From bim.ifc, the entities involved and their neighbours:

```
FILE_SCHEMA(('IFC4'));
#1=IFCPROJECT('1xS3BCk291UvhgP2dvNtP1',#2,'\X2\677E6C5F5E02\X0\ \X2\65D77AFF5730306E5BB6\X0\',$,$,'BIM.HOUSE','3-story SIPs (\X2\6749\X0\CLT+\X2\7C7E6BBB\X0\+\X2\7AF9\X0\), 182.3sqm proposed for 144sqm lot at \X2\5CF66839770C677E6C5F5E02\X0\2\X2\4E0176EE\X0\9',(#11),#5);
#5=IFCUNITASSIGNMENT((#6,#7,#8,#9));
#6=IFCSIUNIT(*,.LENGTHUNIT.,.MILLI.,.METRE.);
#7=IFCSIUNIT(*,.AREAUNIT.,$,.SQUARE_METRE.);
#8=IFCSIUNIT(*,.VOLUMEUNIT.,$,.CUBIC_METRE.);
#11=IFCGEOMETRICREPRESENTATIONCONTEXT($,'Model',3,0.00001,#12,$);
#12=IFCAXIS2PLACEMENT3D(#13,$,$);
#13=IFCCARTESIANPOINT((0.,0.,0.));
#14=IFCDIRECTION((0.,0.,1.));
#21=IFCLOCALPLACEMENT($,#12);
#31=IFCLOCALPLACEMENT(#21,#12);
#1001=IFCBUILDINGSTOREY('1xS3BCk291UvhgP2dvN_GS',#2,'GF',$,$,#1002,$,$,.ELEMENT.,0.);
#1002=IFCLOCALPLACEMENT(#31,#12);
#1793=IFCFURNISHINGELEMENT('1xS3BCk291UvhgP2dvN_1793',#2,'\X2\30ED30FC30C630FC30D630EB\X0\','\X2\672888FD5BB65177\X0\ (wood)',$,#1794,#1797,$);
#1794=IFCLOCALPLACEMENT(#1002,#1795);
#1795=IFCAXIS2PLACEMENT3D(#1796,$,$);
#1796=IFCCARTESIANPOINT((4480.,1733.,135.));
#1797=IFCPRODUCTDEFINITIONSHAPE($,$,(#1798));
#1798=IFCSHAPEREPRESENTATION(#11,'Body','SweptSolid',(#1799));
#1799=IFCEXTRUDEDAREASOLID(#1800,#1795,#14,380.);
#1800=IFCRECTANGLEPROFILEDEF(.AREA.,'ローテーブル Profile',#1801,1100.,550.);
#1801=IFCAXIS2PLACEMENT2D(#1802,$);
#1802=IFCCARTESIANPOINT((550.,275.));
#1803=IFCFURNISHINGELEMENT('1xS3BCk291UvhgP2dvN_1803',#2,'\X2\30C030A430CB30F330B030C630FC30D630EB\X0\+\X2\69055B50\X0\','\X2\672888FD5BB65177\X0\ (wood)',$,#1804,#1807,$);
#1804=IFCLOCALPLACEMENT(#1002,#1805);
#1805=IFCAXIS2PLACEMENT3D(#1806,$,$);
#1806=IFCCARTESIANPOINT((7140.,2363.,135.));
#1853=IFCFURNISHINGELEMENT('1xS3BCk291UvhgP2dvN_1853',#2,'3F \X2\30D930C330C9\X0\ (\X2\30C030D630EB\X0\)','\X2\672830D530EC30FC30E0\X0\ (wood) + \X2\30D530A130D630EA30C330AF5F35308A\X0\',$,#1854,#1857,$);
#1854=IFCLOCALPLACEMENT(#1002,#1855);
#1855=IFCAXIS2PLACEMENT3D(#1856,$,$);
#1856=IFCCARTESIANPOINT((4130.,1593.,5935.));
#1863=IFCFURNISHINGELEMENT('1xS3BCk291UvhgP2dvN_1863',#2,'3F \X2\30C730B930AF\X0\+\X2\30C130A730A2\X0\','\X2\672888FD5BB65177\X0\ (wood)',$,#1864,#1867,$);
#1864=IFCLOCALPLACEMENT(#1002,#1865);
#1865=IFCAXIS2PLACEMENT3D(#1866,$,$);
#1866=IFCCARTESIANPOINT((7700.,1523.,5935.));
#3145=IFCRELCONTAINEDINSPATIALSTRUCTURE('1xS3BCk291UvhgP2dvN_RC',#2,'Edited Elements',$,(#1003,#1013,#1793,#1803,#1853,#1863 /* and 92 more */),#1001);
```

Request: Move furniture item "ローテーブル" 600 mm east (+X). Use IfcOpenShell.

```python
import ifcopenshell
import ifcopenshell.api.geometry
import ifcopenshell.util.placement

model = ifcopenshell.open("bim.ifc")

item = model.by_guid("1xS3BCk291UvhgP2dvN_1793")
matrix = ifcopenshell.util.placement.get_local_placement(item.ObjectPlacement)
matrix[0, 3] += 600.0
ifcopenshell.api.geometry.edit_object_placement(model, product=item, matrix=matrix, is_si=False)

print(ifcopenshell.util.placement.get_local_placement(item.ObjectPlacement).round(3) + 0.0)

model.write("bim_rev.ifc")
```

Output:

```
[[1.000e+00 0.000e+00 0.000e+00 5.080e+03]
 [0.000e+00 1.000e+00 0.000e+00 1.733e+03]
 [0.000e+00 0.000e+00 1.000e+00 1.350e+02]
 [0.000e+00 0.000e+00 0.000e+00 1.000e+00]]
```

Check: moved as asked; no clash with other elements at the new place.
